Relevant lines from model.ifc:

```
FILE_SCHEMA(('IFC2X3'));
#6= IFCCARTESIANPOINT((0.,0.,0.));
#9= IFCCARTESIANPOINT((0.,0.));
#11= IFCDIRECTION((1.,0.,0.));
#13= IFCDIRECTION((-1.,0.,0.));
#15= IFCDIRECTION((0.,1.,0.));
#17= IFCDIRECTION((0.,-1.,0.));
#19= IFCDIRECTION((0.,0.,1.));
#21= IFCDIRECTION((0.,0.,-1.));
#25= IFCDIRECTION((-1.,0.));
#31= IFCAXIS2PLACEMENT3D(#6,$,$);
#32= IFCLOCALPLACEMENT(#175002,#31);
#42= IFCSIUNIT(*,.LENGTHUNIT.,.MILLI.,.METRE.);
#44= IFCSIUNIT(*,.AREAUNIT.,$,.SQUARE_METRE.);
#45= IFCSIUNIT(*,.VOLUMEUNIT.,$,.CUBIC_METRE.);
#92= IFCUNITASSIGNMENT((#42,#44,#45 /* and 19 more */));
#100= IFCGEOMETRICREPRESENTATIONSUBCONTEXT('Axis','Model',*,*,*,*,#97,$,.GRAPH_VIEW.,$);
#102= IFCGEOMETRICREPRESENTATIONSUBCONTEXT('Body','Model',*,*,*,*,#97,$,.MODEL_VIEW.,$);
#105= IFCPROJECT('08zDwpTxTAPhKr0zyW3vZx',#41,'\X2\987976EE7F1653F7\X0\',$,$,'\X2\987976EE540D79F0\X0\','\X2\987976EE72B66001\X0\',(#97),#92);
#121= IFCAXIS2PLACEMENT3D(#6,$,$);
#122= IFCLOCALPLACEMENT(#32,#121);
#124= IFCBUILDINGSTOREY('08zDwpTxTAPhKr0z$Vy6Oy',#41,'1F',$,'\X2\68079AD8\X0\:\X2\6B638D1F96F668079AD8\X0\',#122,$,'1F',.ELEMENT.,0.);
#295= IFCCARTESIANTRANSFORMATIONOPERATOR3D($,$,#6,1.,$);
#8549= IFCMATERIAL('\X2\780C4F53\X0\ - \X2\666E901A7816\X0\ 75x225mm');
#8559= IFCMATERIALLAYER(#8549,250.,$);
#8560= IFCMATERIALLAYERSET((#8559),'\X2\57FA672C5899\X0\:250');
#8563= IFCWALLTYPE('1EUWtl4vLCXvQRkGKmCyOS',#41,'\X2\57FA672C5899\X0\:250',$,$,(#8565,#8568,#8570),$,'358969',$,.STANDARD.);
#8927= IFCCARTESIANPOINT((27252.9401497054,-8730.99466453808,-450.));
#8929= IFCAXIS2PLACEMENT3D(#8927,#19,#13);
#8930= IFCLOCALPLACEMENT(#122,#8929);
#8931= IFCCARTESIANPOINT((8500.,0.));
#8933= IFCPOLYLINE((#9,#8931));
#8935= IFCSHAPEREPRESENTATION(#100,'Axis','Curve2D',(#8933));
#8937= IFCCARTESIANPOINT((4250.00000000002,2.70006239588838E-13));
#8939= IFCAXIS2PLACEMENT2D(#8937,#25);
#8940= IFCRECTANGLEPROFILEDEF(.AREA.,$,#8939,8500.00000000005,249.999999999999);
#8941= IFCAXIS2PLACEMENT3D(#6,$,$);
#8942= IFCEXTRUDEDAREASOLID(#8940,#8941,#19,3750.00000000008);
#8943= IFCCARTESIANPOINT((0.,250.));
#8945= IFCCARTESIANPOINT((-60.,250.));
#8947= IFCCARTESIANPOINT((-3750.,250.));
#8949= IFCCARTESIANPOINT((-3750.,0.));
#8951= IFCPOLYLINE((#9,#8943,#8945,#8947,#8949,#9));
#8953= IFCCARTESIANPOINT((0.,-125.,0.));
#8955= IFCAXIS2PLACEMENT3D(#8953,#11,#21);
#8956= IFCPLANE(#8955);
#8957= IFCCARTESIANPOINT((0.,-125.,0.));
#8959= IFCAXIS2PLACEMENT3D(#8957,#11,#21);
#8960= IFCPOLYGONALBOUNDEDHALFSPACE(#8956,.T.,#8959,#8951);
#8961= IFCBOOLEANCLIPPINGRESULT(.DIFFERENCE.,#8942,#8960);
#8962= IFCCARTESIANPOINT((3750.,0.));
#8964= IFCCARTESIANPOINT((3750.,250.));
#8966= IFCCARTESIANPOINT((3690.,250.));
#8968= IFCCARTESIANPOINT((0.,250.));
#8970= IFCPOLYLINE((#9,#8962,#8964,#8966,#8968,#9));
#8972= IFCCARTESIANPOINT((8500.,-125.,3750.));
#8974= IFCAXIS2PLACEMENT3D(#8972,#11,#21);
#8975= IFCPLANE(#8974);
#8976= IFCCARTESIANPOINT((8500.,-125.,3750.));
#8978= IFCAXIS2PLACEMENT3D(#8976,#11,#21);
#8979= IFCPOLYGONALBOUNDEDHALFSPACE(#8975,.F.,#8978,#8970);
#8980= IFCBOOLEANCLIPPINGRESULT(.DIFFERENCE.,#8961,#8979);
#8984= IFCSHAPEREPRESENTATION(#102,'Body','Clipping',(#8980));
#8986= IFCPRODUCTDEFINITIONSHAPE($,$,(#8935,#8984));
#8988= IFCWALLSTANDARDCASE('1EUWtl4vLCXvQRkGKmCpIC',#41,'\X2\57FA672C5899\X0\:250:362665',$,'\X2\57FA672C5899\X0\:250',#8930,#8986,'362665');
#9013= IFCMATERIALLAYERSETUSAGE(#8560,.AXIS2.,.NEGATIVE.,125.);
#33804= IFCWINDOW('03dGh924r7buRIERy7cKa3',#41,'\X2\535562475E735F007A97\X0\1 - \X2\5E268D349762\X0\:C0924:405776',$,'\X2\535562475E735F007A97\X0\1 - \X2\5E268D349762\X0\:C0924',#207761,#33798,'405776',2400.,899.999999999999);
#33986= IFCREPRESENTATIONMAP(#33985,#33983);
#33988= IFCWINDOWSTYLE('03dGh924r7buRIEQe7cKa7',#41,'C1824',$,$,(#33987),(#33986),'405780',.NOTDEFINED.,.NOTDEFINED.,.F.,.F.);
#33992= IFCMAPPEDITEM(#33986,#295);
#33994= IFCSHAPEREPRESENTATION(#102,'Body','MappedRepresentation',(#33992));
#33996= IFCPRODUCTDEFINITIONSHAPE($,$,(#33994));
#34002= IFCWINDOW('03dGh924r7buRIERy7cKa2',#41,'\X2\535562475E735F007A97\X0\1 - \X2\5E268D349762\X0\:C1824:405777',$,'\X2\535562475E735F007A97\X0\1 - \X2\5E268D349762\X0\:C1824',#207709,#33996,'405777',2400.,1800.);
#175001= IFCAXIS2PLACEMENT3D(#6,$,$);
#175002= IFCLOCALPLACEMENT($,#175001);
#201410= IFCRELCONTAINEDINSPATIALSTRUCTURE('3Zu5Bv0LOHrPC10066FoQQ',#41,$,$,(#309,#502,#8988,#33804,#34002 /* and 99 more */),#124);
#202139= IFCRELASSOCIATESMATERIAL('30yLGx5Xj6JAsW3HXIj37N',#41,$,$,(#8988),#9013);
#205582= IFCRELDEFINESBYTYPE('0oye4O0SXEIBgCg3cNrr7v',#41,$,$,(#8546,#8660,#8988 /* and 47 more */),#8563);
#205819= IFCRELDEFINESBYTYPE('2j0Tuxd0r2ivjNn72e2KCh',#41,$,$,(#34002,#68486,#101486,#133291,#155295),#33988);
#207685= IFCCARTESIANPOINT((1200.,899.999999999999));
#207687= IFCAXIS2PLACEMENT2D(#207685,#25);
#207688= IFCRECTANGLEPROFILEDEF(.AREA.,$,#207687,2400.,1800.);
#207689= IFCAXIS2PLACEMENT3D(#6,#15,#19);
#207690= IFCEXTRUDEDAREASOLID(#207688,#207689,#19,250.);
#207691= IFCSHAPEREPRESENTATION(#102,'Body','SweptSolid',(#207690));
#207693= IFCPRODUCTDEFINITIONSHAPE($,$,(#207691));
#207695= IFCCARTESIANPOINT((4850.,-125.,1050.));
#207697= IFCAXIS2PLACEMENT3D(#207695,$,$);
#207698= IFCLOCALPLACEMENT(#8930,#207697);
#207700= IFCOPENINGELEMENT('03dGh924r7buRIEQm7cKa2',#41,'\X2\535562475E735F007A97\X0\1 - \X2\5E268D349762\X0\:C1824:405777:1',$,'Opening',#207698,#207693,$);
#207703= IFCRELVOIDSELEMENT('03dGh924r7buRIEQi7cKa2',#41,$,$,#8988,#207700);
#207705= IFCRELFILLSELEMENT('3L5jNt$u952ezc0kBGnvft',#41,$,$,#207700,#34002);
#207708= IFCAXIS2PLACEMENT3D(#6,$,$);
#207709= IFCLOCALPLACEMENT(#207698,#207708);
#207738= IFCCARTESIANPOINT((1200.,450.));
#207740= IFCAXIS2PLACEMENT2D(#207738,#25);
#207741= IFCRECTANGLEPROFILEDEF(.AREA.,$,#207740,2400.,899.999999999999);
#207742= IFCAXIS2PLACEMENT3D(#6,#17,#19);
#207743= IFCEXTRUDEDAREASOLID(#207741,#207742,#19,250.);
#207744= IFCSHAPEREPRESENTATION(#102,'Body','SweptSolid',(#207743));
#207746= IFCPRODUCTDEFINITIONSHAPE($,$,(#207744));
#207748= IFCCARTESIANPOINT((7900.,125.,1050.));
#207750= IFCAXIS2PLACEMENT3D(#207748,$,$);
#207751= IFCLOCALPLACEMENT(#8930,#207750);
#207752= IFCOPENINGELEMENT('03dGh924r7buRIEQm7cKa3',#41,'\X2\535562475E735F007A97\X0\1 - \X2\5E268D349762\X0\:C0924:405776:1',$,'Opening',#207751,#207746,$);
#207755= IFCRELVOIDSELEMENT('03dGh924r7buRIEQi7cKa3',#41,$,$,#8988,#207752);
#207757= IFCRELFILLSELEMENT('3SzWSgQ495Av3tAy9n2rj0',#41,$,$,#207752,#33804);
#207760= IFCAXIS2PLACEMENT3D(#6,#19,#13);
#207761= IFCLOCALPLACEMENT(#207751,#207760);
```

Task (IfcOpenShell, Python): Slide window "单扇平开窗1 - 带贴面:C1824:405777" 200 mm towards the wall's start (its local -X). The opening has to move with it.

```python
import ifcopenshell
import ifcopenshell.api.geometry
import ifcopenshell.util.placement

model = ifcopenshell.open("model.ifc")

window = model.by_id(34002)
opening = window.FillsVoids[0].RelatingOpeningElement
wall = opening.VoidsElements[0].RelatingBuildingElement

wall_matrix = ifcopenshell.util.placement.get_local_placement(wall.ObjectPlacement)
shift = wall_matrix[:3, 0] * -200.0
before = ifcopenshell.util.placement.get_local_placement(window.ObjectPlacement)[:3, 3].copy()

# The window is placed relative to its opening, so it follows when the opening moves.
matrix = ifcopenshell.util.placement.get_local_placement(opening.ObjectPlacement)
matrix[:3, 3] += shift
ifcopenshell.api.geometry.edit_object_placement(
    model, product=opening, matrix=matrix, is_si=False, should_transform_children=True
)

after = ifcopenshell.util.placement.get_local_placement(window.ObjectPlacement)[:3, 3]
print("window moved by", (after - before).round(3) + 0.0)

model.write("model_edited.ifc")
```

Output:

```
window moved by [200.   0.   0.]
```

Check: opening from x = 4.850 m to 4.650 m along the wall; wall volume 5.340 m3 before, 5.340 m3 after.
